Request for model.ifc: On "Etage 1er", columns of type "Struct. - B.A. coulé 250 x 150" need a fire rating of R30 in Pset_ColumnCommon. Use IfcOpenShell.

First a look at what the model holds.

```python
import ifcopenshell
import ifcopenshell.util.element

model = ifcopenshell.open("model.ifc")
print(model.schema)
storey = next(s for s in model.by_type("IfcBuildingStorey") if s.Name == "Etage 1er")
columns = [e for e in ifcopenshell.util.element.get_decomposition(storey) if e.is_a("IfcColumn")]
seen = {}
for e in columns:
    element_type = ifcopenshell.util.element.get_type(e)
    key = (element_type.Name if element_type != e and element_type else None, ifcopenshell.util.element.get_pset(e, "Pset_ColumnCommon", "FireRating"))
    seen[key] = seen.get(key, 0) + 1
for (name, value), count in sorted(seen.items(), key=str):
    print(count, "x", name, "|", value)
```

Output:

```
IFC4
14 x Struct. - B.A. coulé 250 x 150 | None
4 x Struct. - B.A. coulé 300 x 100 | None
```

```python
import ifcopenshell
import ifcopenshell.api.pset
import ifcopenshell.util.element

model = ifcopenshell.open("model.ifc")

storey = next(s for s in model.by_type("IfcBuildingStorey") if s.Name == "Etage 1er")
columns = [e for e in ifcopenshell.util.element.get_decomposition(storey) if e.is_a("IfcColumn")]

count = 0
for e in columns:
    element_type = ifcopenshell.util.element.get_type(e)
    if element_type in (None, e) or element_type.Name != "Struct. - B.A. coulé 250 x 150":
        continue
    # add_pset returns the element's existing set when there is one.
    pset = ifcopenshell.api.pset.add_pset(model, product=e, name="Pset_ColumnCommon")
    ifcopenshell.api.pset.edit_pset(model, pset=pset, properties={"FireRating": "R30"})
    count += 1

print(count, "columns updated")

model.write("model_rev.ifc")
```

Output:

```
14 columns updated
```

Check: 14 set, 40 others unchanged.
